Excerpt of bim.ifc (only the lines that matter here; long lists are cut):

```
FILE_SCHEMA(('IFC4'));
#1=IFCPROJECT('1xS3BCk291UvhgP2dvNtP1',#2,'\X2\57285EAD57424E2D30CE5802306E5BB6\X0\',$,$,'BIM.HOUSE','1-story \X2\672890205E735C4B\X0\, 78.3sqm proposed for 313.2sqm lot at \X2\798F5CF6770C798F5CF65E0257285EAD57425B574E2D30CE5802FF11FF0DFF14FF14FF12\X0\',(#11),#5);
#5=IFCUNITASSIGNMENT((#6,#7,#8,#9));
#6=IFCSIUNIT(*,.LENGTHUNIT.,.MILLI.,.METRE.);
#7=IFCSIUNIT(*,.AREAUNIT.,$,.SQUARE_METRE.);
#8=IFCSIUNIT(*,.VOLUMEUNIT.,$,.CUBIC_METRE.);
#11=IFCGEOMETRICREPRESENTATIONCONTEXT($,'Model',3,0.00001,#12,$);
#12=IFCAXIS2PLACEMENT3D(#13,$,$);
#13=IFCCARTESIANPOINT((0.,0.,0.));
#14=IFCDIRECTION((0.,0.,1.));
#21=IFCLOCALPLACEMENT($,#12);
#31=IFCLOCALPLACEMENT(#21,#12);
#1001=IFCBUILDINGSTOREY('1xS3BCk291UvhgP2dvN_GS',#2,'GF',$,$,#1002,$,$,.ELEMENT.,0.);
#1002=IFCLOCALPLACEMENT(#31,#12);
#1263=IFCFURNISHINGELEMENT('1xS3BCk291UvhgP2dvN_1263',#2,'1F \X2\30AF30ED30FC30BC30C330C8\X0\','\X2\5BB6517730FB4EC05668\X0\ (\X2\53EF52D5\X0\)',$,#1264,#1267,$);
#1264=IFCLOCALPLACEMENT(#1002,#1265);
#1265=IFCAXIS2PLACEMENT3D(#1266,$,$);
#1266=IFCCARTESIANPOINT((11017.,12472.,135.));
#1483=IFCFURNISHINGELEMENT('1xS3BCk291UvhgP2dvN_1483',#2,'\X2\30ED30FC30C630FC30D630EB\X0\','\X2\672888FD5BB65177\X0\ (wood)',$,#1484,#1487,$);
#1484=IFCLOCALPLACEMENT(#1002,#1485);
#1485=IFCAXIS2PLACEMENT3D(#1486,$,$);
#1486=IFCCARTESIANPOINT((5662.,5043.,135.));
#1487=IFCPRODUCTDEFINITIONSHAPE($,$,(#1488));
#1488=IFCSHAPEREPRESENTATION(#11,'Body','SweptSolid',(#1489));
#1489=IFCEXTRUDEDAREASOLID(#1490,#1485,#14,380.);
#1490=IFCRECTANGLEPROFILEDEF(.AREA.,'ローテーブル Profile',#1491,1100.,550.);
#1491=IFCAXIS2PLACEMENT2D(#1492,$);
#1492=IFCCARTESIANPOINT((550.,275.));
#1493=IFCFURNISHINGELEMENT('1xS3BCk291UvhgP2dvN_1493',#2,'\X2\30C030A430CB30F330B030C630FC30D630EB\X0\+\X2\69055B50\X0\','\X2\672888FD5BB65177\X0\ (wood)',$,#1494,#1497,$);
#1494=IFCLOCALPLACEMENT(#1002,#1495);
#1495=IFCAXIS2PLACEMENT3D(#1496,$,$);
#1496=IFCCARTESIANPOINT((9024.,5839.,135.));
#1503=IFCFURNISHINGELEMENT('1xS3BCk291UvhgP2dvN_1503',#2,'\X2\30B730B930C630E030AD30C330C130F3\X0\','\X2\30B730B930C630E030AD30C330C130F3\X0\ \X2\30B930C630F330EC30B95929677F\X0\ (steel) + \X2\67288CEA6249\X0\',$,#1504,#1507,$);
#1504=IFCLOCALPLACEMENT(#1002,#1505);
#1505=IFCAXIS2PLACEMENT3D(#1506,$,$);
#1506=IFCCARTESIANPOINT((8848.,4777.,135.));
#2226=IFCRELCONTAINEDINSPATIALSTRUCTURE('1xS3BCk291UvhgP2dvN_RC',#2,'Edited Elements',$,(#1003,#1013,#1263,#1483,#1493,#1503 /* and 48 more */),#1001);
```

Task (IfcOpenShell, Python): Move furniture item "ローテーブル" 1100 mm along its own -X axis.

```python
import ifcopenshell
import ifcopenshell.api.geometry
import ifcopenshell.util.placement

model = ifcopenshell.open("bim.ifc")

item = model.by_guid("1xS3BCk291UvhgP2dvN_1483")
matrix = ifcopenshell.util.placement.get_local_placement(item.ObjectPlacement)
matrix[:3, 3] -= matrix[:3, 0] * 1100.0
ifcopenshell.api.geometry.edit_object_placement(model, product=item, matrix=matrix, is_si=False)

print(ifcopenshell.util.placement.get_local_placement(item.ObjectPlacement).round(3) + 0.0)

model.write("bim_rev.ifc")
```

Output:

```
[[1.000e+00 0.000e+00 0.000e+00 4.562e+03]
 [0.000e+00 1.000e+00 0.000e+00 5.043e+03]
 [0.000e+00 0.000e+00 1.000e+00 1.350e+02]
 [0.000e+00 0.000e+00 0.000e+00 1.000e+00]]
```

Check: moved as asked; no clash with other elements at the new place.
